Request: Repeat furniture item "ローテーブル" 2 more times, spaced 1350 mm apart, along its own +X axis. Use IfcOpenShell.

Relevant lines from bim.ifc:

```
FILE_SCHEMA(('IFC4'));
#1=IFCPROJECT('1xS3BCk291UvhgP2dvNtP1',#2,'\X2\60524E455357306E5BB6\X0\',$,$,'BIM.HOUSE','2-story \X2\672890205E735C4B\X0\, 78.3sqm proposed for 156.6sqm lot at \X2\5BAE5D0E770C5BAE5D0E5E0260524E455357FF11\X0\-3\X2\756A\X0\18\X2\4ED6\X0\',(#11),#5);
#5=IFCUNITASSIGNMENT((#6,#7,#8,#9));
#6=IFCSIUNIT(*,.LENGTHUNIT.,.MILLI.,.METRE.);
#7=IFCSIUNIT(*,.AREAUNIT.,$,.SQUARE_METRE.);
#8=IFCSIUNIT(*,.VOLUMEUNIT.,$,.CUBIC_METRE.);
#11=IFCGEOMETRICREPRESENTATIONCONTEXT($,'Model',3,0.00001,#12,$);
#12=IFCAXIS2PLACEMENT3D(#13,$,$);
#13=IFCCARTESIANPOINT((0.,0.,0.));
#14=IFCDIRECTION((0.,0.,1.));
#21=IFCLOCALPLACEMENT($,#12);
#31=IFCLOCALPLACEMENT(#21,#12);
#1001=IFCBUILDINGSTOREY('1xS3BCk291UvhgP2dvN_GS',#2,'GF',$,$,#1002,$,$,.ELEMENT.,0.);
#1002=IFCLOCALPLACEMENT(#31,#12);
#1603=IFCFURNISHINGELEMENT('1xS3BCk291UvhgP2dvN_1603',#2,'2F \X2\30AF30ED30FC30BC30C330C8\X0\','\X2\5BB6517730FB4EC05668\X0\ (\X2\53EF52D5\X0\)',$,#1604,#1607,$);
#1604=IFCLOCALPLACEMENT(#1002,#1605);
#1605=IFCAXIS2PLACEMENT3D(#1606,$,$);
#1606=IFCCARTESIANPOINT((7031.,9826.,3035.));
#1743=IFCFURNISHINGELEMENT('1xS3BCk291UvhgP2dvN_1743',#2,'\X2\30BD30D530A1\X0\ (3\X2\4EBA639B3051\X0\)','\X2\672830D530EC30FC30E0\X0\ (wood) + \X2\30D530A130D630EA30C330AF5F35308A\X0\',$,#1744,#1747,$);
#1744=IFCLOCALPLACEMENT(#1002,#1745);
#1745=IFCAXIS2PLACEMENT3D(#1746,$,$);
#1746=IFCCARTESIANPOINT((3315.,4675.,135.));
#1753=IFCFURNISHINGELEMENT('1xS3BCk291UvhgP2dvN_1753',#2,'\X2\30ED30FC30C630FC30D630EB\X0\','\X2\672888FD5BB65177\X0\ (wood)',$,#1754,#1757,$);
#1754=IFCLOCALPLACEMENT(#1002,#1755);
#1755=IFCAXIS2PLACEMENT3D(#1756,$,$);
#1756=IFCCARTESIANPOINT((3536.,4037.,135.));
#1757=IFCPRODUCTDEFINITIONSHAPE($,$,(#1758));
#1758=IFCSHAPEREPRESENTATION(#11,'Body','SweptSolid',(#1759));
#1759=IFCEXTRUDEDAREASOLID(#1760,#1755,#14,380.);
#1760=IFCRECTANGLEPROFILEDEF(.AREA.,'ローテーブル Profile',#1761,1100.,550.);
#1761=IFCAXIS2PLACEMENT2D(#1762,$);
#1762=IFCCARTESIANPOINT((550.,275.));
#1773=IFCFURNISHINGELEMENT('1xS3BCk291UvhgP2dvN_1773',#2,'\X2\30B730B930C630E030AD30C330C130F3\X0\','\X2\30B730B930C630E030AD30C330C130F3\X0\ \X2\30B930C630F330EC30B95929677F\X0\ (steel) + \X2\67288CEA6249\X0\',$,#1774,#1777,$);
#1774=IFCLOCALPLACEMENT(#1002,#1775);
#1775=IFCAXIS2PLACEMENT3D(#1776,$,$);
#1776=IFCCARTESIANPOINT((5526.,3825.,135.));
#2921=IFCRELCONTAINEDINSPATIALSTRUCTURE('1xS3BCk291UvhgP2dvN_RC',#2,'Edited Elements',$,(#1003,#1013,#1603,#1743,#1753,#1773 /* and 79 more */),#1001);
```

```python
import ifcopenshell
import ifcopenshell.api.geometry
import ifcopenshell.api.root
import ifcopenshell.util.element
import ifcopenshell.util.placement
import ifcopenshell.util.unit

model = ifcopenshell.open("bim.ifc")
unit_scale = ifcopenshell.util.unit.calculate_unit_scale(model)


def reuse_history(source, copy):
    """copy_class also copies each property set's owner history, people and application; keep the originals."""
    for rel in copy.IsDefinedBy:
        if rel.is_a("IfcRelDefinesByProperties") and (history := rel.RelatingPropertyDefinition.OwnerHistory):
            rel.RelatingPropertyDefinition.OwnerHistory = source.OwnerHistory
            ifcopenshell.util.element.remove_deep2(model, history)


source = model.by_guid("1xS3BCk291UvhgP2dvN_1753")
base = ifcopenshell.util.placement.get_local_placement(source.ObjectPlacement)
step = base[:3, 0] * 1.35 / unit_scale

for i in range(1, 3):
    copy = ifcopenshell.api.root.copy_class(model, product=source)
    copy.Representation = ifcopenshell.util.element.copy_deep(
        model, source.Representation, exclude=["IfcGeometricRepresentationContext", "IfcRepresentationMap"]
    )
    reuse_history(source, copy)
    matrix = base.copy()
    matrix[:3, 3] += i * step
    print("added at", matrix[:3, 3].round(3) + 0.0)
    ifcopenshell.api.geometry.edit_object_placement(model, product=copy, matrix=matrix, is_si=False)

model.write("bim_updated.ifc")
```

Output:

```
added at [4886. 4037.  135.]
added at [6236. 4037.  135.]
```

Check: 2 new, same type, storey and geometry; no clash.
